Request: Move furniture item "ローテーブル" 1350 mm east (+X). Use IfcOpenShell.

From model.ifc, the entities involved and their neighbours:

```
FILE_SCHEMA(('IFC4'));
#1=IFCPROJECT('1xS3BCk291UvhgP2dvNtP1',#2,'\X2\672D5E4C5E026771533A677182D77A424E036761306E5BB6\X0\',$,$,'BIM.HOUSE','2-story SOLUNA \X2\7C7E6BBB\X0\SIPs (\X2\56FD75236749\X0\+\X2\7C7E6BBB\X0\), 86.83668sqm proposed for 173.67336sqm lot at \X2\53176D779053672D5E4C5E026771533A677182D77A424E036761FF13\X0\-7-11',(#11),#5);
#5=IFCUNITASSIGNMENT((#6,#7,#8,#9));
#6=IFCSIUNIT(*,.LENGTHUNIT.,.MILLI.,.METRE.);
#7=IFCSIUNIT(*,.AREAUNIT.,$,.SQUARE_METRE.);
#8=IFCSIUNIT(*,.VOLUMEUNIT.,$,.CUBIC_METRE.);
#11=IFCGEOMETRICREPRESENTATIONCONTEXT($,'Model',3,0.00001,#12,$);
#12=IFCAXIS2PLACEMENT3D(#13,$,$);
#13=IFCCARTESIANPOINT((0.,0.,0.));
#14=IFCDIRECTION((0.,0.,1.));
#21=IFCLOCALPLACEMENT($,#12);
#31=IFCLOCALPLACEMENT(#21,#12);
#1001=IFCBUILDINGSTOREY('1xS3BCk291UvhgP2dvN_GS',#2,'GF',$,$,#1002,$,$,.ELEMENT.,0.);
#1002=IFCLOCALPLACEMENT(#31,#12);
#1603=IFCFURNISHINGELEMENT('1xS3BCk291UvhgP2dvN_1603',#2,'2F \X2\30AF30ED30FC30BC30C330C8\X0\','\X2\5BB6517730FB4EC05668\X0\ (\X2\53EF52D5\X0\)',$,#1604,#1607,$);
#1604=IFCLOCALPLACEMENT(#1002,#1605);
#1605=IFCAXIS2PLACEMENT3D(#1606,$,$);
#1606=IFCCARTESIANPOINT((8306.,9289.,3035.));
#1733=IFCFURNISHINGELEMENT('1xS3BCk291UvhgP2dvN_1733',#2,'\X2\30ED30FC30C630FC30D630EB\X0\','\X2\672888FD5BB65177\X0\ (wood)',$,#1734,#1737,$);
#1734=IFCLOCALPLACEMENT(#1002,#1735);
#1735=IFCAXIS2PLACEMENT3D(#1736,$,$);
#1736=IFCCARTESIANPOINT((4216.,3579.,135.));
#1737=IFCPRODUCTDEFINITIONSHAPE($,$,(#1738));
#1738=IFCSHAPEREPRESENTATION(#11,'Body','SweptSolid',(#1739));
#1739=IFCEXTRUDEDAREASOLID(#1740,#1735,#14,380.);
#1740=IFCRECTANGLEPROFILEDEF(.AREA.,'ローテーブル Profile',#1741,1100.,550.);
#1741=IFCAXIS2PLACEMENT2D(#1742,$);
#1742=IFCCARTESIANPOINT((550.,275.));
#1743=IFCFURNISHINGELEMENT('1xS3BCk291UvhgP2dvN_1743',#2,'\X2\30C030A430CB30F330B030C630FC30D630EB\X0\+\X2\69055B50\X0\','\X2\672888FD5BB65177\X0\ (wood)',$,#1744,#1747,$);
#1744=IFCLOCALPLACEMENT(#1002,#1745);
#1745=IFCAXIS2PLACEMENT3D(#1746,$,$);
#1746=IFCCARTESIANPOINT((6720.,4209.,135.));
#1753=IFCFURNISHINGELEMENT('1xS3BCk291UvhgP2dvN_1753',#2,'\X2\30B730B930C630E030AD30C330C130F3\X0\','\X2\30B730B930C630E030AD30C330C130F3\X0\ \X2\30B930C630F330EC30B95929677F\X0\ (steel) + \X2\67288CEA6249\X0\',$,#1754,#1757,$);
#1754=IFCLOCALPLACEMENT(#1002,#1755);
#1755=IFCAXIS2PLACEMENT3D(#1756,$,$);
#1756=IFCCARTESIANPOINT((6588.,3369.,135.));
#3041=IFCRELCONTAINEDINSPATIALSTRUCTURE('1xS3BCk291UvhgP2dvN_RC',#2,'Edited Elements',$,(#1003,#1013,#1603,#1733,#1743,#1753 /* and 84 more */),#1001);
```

```python
import ifcopenshell
import ifcopenshell.api.geometry
import ifcopenshell.util.placement
import ifcopenshell.util.unit

model = ifcopenshell.open("model.ifc")
unit_scale = ifcopenshell.util.unit.calculate_unit_scale(model)

item = model.by_guid("1xS3BCk291UvhgP2dvN_1733")
matrix = ifcopenshell.util.placement.get_local_placement(item.ObjectPlacement)
matrix[0, 3] += 1.35 / unit_scale
ifcopenshell.api.geometry.edit_object_placement(model, product=item, matrix=matrix, is_si=False)

print(ifcopenshell.util.placement.get_local_placement(item.ObjectPlacement).round(3) + 0.0)

model.write("model_rev.ifc")
```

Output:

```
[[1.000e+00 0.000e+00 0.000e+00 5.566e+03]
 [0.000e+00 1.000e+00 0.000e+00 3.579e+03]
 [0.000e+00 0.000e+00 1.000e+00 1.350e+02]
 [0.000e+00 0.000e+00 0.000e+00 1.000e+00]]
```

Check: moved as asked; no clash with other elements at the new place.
